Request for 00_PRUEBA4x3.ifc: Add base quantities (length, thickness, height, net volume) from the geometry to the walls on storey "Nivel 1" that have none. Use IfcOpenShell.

First a look at what the model holds.

```python
import ifcopenshell
import ifcopenshell.util.element
import ifcopenshell.util.unit

model = ifcopenshell.open("00_PRUEBA4x3.ifc")
print(model.schema)
for unit_type in ("LENGTHUNIT", "AREAUNIT", "VOLUMEUNIT"):
    print(unit_type, ifcopenshell.util.unit.calculate_unit_scale(model, unit_type))
storey = next(s for s in model.by_type("IfcBuildingStorey") if s.Name == "Nivel 1")
walls = [e for e in ifcopenshell.util.element.get_decomposition(storey) if e.is_a("IfcWall")]
for e in sorted(walls, key=lambda e: e.id()):
    print(e.id(), e.is_a(), e.Name, list(ifcopenshell.util.element.get_psets(e, qtos_only=True)), sep=" | ")
```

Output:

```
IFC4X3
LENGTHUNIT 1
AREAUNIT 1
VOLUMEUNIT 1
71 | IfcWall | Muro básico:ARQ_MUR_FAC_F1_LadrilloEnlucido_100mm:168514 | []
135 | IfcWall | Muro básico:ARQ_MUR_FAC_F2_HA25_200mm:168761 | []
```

```python
import ifcopenshell
import ifcopenshell.api.pset
import ifcopenshell.geom
import ifcopenshell.util.element
import ifcopenshell.util.shape
import ifcopenshell.util.unit

model = ifcopenshell.open("00_PRUEBA4x3.ifc")
unit_scale = ifcopenshell.util.unit.calculate_unit_scale(model)
volume_scale = ifcopenshell.util.unit.calculate_unit_scale(model, "VOLUMEUNIT")
settings = ifcopenshell.geom.settings()

storey = next(s for s in model.by_type("IfcBuildingStorey") if s.Name == "Nivel 1")
walls = [e for e in ifcopenshell.util.element.get_decomposition(storey) if e.is_a("IfcWall")]

for e in sorted(walls, key=lambda e: e.id()):
    if ifcopenshell.util.element.get_psets(e, qtos_only=True, should_inherit=False):
        continue
    # Geometry comes back in metres, in the element's own axes.
    shape = ifcopenshell.geom.create_shape(settings, e)
    values = {
        "Length": ifcopenshell.util.shape.get_x(shape.geometry) / unit_scale,
        "Width": ifcopenshell.util.shape.get_y(shape.geometry) / unit_scale,
        "Height": ifcopenshell.util.shape.get_z(shape.geometry) / unit_scale,
        "NetVolume": ifcopenshell.util.shape.get_volume(shape.geometry) / volume_scale,
    }
    qto = ifcopenshell.api.pset.add_qto(model, product=e, name="Qto_WallBaseQuantities")
    ifcopenshell.api.pset.edit_qto(model, qto=qto, properties=values)
    print(e.id(), {k: round(v, 3) for k, v in values.items()})

model.write("00_PRUEBA4x3_edited.ifc")
```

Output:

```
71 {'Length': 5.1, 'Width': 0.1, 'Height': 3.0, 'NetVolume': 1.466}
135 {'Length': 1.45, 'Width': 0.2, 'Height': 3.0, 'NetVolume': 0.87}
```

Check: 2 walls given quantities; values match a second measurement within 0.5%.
